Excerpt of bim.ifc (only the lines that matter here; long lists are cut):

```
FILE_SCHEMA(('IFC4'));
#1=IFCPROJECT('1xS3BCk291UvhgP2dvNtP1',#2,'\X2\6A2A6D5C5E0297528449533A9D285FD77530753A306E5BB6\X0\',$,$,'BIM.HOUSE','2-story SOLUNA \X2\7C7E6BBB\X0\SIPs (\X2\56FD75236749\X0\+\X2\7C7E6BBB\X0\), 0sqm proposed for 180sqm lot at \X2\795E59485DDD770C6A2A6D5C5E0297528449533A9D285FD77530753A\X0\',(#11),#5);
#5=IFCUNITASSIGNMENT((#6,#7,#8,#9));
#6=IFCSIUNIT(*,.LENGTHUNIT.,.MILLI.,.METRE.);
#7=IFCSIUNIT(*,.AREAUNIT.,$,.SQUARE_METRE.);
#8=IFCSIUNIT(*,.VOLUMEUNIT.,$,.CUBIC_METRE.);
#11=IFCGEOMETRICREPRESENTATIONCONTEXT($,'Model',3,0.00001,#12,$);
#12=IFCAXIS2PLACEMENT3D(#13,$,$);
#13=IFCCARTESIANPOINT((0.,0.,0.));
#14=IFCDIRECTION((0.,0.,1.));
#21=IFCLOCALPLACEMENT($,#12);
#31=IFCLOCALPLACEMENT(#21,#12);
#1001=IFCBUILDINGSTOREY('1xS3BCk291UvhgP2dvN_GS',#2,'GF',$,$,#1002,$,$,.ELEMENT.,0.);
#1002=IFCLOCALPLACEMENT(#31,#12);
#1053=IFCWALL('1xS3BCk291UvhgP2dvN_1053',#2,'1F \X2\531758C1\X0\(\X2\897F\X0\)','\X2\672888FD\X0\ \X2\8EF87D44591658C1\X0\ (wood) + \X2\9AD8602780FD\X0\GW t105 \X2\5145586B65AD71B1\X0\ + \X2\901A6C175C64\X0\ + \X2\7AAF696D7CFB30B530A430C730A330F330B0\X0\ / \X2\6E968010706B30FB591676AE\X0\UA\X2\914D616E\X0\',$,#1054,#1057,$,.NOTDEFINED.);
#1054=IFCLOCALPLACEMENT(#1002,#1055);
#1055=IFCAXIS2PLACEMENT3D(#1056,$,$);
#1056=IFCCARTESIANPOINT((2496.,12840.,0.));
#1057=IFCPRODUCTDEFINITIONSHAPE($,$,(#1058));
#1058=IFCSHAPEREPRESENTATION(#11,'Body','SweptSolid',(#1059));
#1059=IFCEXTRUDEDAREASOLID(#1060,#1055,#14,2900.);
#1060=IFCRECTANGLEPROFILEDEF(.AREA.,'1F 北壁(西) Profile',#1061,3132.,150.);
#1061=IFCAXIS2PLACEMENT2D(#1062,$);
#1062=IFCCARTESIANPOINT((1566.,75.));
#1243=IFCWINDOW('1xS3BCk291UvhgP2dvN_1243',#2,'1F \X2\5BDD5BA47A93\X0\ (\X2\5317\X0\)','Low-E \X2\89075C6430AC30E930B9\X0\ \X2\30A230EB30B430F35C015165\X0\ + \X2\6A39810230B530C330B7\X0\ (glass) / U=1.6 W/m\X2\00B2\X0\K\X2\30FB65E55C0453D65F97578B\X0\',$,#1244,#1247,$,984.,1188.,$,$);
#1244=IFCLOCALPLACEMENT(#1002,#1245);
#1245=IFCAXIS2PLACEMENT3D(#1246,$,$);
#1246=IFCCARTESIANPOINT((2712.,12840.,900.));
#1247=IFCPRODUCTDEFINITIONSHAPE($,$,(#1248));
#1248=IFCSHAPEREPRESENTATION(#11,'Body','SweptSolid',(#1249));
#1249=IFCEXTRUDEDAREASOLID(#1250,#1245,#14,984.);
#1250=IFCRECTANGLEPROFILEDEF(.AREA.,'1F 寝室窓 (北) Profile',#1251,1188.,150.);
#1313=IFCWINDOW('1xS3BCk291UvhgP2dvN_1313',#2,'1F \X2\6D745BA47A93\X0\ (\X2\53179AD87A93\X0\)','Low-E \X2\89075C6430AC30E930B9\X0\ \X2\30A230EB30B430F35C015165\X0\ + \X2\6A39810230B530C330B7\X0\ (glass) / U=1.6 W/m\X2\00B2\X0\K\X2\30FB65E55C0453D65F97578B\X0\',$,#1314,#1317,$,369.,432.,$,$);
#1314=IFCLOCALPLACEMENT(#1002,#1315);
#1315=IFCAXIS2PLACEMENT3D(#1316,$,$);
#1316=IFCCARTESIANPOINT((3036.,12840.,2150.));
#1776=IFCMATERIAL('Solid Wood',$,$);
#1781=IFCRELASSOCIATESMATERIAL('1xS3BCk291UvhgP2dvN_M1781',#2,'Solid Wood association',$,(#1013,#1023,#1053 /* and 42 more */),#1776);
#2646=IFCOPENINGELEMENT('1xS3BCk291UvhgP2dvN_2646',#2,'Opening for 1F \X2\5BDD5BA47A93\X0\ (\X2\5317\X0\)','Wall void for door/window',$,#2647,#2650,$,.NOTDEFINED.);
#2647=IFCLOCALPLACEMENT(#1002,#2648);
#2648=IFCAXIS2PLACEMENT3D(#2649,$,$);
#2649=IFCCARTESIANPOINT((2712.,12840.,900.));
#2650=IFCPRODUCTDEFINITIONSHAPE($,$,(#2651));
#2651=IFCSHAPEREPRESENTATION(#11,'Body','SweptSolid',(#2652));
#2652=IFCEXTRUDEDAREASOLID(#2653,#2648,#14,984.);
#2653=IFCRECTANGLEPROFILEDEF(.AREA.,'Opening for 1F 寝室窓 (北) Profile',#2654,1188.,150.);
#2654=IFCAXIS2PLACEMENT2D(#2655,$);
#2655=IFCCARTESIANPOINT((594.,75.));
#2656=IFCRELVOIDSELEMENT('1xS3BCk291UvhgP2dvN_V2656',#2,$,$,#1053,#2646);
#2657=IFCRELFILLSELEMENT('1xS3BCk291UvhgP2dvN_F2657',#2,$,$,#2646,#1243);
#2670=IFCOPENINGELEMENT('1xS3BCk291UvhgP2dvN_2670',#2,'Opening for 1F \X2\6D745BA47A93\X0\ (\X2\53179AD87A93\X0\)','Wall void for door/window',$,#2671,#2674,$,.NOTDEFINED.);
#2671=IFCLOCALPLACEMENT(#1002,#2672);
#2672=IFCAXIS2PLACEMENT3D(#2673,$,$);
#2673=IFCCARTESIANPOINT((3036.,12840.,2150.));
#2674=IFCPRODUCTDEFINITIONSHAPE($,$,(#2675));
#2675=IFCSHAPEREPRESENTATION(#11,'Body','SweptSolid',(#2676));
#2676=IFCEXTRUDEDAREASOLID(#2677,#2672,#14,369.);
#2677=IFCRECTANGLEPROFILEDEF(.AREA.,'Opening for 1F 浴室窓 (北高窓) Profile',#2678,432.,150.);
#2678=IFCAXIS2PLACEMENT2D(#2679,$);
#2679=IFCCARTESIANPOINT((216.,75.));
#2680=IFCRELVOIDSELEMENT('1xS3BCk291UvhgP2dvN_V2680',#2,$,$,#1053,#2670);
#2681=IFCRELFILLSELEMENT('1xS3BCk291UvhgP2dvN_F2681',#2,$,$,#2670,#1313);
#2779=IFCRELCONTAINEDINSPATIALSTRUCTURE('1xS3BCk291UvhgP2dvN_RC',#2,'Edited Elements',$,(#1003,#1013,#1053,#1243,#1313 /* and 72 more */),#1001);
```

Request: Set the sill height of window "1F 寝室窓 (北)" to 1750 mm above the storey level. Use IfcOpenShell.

```python
import numpy as np
import ifcopenshell
import ifcopenshell.api.geometry
import ifcopenshell.geom
import ifcopenshell.util.element
import ifcopenshell.util.placement
import ifcopenshell.util.shape
import ifcopenshell.util.unit

model = ifcopenshell.open("bim.ifc")
unit_scale = ifcopenshell.util.unit.calculate_unit_scale(model)

window = model.by_guid("1xS3BCk291UvhgP2dvN_1243")
opening = window.FillsVoids[0].RelatingOpeningElement
storey = ifcopenshell.util.element.get_container(window, ifc_class="IfcBuildingStorey")
level = ifcopenshell.util.placement.get_local_placement(storey.ObjectPlacement)[2, 3]

# The opening's origin need not be at the sill, so measure its lowest point.
shape = ifcopenshell.geom.create_shape(ifcopenshell.geom.settings(), opening)
bottom = ifcopenshell.util.shape.get_shape_bottom_elevation(shape, shape.geometry) / unit_scale
dz = level + 1.75 / unit_scale - bottom

shift = np.array([0.0, 0.0, dz])
# The window is not placed relative to its opening, so move both.
for product in (opening, window):
    matrix = ifcopenshell.util.placement.get_local_placement(product.ObjectPlacement)
    matrix[:3, 3] += shift
    ifcopenshell.api.geometry.edit_object_placement(model, product=product, matrix=matrix, is_si=False)

print(f"moved by {dz * unit_scale:+.3f} m")

model.write("bim_edited.ifc")
```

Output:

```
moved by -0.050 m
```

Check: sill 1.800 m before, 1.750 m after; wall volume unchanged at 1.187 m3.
